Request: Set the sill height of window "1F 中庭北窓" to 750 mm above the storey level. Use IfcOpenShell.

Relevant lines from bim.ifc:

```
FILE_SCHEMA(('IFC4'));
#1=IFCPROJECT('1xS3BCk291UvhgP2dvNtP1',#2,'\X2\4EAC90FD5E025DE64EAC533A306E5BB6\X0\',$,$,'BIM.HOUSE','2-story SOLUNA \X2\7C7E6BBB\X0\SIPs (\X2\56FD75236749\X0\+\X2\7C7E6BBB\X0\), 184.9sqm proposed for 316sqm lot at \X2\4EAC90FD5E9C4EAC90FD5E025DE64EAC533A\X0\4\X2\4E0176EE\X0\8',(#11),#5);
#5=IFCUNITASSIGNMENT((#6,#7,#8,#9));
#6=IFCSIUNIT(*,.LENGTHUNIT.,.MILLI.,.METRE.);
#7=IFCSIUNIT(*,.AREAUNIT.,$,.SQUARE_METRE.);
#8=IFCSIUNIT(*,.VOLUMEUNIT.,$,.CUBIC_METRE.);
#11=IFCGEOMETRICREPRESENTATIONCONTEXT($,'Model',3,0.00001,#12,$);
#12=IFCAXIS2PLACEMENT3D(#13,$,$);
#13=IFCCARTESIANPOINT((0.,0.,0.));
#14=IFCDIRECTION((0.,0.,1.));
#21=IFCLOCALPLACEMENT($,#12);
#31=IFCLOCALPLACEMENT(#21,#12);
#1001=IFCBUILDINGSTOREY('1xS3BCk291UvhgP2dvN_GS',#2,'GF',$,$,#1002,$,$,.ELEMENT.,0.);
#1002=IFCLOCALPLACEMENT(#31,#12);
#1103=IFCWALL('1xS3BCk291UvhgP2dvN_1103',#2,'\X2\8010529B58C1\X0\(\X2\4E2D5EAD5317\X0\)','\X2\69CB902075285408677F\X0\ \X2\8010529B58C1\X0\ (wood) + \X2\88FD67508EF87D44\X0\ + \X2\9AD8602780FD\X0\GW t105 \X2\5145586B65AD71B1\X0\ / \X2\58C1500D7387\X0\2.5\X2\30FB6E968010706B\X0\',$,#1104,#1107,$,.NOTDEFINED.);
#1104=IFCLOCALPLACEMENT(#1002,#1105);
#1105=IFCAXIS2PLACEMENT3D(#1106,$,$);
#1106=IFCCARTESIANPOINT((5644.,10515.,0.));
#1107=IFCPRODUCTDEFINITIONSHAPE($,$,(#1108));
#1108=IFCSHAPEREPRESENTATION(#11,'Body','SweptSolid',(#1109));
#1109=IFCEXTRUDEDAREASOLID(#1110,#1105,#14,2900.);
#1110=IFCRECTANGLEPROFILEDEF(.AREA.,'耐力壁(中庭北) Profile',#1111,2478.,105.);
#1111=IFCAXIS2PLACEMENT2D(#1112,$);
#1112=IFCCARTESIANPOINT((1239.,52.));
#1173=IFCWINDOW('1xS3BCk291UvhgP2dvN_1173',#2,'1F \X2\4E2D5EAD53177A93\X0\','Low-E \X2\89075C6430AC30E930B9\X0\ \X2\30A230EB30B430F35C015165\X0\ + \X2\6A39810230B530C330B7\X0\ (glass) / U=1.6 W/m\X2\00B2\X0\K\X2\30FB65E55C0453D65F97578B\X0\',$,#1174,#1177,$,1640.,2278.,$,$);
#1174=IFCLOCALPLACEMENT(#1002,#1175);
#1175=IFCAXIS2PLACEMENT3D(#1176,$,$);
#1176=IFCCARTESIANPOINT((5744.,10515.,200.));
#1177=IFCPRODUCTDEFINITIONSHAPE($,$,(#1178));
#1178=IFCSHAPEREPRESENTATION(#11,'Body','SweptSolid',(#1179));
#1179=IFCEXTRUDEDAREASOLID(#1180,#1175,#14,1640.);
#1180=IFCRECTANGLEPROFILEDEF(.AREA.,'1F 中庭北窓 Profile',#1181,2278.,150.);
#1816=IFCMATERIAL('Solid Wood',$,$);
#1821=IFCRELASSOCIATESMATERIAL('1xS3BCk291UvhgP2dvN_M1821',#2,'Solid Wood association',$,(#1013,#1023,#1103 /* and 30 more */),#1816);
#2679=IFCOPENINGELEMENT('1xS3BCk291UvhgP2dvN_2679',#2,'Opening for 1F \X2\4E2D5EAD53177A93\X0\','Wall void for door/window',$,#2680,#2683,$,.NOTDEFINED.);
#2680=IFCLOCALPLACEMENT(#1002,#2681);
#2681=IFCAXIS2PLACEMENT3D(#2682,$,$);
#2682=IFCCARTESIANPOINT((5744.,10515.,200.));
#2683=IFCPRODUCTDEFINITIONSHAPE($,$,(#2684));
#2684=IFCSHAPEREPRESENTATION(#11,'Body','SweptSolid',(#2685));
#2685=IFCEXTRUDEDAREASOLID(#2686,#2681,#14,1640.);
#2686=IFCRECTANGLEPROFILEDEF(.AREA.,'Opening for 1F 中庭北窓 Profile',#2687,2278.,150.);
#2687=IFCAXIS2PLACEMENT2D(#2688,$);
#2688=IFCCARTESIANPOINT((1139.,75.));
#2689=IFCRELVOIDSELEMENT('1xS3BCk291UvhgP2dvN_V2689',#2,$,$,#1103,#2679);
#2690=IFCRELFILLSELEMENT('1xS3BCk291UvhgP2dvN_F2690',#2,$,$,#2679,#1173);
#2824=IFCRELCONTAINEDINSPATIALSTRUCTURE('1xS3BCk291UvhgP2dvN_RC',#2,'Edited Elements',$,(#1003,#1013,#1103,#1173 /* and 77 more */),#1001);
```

```python
import numpy as np
import ifcopenshell
import ifcopenshell.api.geometry
import ifcopenshell.geom
import ifcopenshell.util.element
import ifcopenshell.util.placement
import ifcopenshell.util.shape
import ifcopenshell.util.unit

model = ifcopenshell.open("bim.ifc")
unit_scale = ifcopenshell.util.unit.calculate_unit_scale(model)

window = model.by_guid("1xS3BCk291UvhgP2dvN_1173")
opening = window.FillsVoids[0].RelatingOpeningElement
storey = ifcopenshell.util.element.get_container(window, ifc_class="IfcBuildingStorey")
level = ifcopenshell.util.placement.get_local_placement(storey.ObjectPlacement)[2, 3]

# The opening's origin need not be at the sill, so measure its lowest point.
shape = ifcopenshell.geom.create_shape(ifcopenshell.geom.settings(), opening)
bottom = ifcopenshell.util.shape.get_shape_bottom_elevation(shape, shape.geometry) / unit_scale
dz = level + 750.0 - bottom

shift = np.array([0.0, 0.0, dz])
# The window is not placed relative to its opening, so move both.
for product in (opening, window):
    matrix = ifcopenshell.util.placement.get_local_placement(product.ObjectPlacement)
    matrix[:3, 3] += shift
    ifcopenshell.api.geometry.edit_object_placement(model, product=product, matrix=matrix, is_si=False)

print(f"moved by {dz * unit_scale:+.3f} m")

model.write("bim-out.ifc")
```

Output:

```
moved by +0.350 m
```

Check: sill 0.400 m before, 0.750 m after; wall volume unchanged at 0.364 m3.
